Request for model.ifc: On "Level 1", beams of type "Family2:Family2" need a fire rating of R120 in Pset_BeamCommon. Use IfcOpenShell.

First a look at what the model holds.

```python
import ifcopenshell
import ifcopenshell.util.element

model = ifcopenshell.open("model.ifc")
print(model.schema)
storey = next(s for s in model.by_type("IfcBuildingStorey") if s.Name == "Level 1")
beams = [e for e in ifcopenshell.util.element.get_decomposition(storey) if e.is_a("IfcBeam")]
seen = {}
for e in beams:
    element_type = ifcopenshell.util.element.get_type(e)
    key = (element_type.Name if element_type != e and element_type else None, ifcopenshell.util.element.get_pset(e, "Pset_BeamCommon", "FireRating"))
    seen[key] = seen.get(key, 0) + 1
for (name, value), count in sorted(seen.items(), key=str):
    print(count, "x", name, "|", value)
```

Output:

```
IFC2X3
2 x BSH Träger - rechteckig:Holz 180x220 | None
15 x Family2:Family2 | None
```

```python
import ifcopenshell
import ifcopenshell.api.pset
import ifcopenshell.util.element

model = ifcopenshell.open("model.ifc")

storey = next(s for s in model.by_type("IfcBuildingStorey") if s.Name == "Level 1")
beams = [e for e in ifcopenshell.util.element.get_decomposition(storey) if e.is_a("IfcBeam")]

count = 0
for e in beams:
    element_type = ifcopenshell.util.element.get_type(e)
    if element_type in (None, e) or element_type.Name != "Family2:Family2":
        continue
    # add_pset returns the element's existing set when there is one.
    pset = ifcopenshell.api.pset.add_pset(model, product=e, name="Pset_BeamCommon")
    ifcopenshell.api.pset.edit_pset(model, pset=pset, properties={"FireRating": "R120"})
    count += 1

print(count, "beams updated")

model.write("model_v2.ifc")
```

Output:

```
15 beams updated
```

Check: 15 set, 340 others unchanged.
